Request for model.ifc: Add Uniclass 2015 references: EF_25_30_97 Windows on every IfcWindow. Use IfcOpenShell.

First a look at what the model holds.

```python
import ifcopenshell

model = ifcopenshell.open("model.ifc")
print(model.schema)
print("classifications:", [c.Name for c in model.by_type("IfcClassification")])
for ifc_class in ("IfcDoor", "IfcRoof", "IfcStair", "IfcWall", "IfcWindow"):
    print(ifc_class, len(model.by_type(ifc_class)))
```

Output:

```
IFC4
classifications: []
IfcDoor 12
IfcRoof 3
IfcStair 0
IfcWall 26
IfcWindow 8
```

```python
import ifcopenshell
import ifcopenshell.api.classification

model = ifcopenshell.open("model.ifc")

system = ifcopenshell.api.classification.add_classification(model, classification="Uniclass 2015")

codes = {
    "IfcWindow": ("EF_25_30_97", "Windows"),
}
for ifc_class, (code, name) in codes.items():
    products = model.by_type(ifc_class)
    ifcopenshell.api.classification.add_reference(
        model, products=products, classification=system, identification=code, name=name
    )
    print(code, len(products))

model.write("model_updated.ifc")
```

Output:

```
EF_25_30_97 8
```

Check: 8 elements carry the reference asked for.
